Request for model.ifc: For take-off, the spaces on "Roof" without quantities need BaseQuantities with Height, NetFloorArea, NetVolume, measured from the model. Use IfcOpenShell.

First a look at what the model holds.

```python
import ifcopenshell
import ifcopenshell.util.element
import ifcopenshell.util.unit

model = ifcopenshell.open("model.ifc")
print(model.schema)
for unit_type in ("LENGTHUNIT", "AREAUNIT", "VOLUMEUNIT"):
    print(unit_type, ifcopenshell.util.unit.calculate_unit_scale(model, unit_type))
storey = next(s for s in model.by_type("IfcBuildingStorey") if s.Name == "Roof")
spaces = [e for e in ifcopenshell.util.element.get_decomposition(storey) if e.is_a("IfcSpace")]
for e in sorted(spaces, key=lambda e: e.id()):
    print(e.id(), e.is_a(), e.Name, list(ifcopenshell.util.element.get_psets(e, qtos_only=True)), sep=" | ")
```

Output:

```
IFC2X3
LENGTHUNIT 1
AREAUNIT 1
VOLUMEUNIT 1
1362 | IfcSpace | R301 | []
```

```python
import ifcopenshell
import ifcopenshell.api.pset
import ifcopenshell.geom
import ifcopenshell.util.element
import ifcopenshell.util.shape
import ifcopenshell.util.unit

model = ifcopenshell.open("model.ifc")
unit_scale = ifcopenshell.util.unit.calculate_unit_scale(model)
area_scale = ifcopenshell.util.unit.calculate_unit_scale(model, "AREAUNIT")
volume_scale = ifcopenshell.util.unit.calculate_unit_scale(model, "VOLUMEUNIT")
settings = ifcopenshell.geom.settings()

storey = next(s for s in model.by_type("IfcBuildingStorey") if s.Name == "Roof")
spaces = [e for e in ifcopenshell.util.element.get_decomposition(storey) if e.is_a("IfcSpace")]

for e in sorted(spaces, key=lambda e: e.id()):
    if ifcopenshell.util.element.get_psets(e, qtos_only=True, should_inherit=False):
        continue
    # Geometry comes back in metres, in the element's own axes.
    shape = ifcopenshell.geom.create_shape(settings, e)
    values = {
        "Height": ifcopenshell.util.shape.get_z(shape.geometry) / unit_scale,
        "NetFloorArea": ifcopenshell.util.shape.get_footprint_area(shape.geometry) / area_scale,
        "NetVolume": ifcopenshell.util.shape.get_volume(shape.geometry) / volume_scale,
    }
    qto = ifcopenshell.api.pset.add_qto(model, product=e, name="BaseQuantities")
    ifcopenshell.api.pset.edit_qto(model, qto=qto, properties=values)
    print(e.id(), {k: round(v, 3) for k, v in values.items()})

model.write("model_edited.ifc")
```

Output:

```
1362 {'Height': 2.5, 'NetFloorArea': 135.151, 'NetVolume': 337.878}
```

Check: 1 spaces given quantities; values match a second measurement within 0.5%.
